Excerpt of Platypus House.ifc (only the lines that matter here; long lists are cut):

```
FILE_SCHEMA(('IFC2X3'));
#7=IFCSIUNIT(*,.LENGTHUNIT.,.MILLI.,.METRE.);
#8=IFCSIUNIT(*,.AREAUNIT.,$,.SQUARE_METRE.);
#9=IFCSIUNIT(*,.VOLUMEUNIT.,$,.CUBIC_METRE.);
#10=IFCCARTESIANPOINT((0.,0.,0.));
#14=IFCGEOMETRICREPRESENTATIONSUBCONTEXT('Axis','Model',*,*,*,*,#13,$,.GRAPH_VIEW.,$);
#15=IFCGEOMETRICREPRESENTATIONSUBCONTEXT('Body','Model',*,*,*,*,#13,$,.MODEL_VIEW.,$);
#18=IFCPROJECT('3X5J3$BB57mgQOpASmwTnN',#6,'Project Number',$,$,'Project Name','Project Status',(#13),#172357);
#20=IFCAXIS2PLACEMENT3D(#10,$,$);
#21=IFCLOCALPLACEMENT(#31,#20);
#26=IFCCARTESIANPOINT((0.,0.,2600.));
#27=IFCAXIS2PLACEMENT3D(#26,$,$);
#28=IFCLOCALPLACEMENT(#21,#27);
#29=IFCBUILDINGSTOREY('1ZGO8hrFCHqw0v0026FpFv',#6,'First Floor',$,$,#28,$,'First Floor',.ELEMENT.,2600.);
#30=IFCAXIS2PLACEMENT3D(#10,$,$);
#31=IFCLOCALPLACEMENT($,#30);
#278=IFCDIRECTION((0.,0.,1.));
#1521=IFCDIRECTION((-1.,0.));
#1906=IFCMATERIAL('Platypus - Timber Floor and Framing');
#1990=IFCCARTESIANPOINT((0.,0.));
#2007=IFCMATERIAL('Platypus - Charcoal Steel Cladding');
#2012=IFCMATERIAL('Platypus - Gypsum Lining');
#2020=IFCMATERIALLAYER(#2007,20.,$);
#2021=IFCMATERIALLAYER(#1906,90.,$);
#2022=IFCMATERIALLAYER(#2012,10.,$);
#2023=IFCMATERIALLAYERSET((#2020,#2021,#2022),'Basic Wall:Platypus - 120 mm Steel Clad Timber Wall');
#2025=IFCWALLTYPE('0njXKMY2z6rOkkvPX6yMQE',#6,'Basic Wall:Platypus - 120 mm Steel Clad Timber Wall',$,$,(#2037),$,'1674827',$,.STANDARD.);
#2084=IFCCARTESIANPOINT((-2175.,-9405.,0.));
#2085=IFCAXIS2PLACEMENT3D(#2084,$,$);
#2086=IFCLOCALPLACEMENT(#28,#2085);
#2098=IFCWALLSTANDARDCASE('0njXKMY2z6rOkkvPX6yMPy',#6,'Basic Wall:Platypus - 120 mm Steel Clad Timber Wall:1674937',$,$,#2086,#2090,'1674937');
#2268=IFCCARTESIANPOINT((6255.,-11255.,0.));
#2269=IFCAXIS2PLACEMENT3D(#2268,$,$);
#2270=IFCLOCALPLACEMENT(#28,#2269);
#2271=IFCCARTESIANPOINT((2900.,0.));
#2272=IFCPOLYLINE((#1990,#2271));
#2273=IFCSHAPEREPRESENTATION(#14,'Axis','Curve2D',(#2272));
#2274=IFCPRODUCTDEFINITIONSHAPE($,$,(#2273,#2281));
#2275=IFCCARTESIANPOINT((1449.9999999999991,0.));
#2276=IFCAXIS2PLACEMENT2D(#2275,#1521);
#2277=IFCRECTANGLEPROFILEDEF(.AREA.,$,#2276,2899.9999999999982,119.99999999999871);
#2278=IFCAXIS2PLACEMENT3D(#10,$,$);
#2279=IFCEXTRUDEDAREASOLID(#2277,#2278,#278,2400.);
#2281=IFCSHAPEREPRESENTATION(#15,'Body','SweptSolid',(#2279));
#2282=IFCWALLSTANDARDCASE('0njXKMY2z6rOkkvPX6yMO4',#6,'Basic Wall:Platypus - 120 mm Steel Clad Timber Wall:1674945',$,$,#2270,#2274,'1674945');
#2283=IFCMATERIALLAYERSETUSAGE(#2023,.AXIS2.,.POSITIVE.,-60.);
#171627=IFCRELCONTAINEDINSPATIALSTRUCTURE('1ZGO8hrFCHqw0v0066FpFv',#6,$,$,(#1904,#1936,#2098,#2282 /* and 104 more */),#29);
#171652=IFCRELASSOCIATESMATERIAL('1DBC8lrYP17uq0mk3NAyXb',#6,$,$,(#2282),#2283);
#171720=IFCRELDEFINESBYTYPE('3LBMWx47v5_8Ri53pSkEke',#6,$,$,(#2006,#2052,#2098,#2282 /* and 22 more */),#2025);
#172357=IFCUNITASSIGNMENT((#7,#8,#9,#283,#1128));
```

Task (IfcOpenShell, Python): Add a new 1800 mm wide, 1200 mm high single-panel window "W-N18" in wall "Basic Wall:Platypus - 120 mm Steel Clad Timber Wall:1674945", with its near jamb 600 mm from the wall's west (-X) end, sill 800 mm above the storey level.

```python
import numpy as np
import ifcopenshell
import ifcopenshell.api.feature
import ifcopenshell.api.geometry
import ifcopenshell.api.root
import ifcopenshell.api.spatial
import ifcopenshell.api.type
import ifcopenshell.geom
import ifcopenshell.util.element
import ifcopenshell.util.placement
import ifcopenshell.util.representation
import ifcopenshell.util.shape
import ifcopenshell.util.unit

model = ifcopenshell.open("Platypus House.ifc")
unit_scale = ifcopenshell.util.unit.calculate_unit_scale(model)
settings = ifcopenshell.geom.settings()


def volume(element):
    """Net volume in cubic metres, openings subtracted."""
    shape = ifcopenshell.geom.create_shape(settings, element)
    return ifcopenshell.util.shape.get_volume(shape.geometry)


wall = model.by_guid("0njXKMY2z6rOkkvPX6yMO4")
storey = ifcopenshell.util.element.get_container(wall, ifc_class="IfcBuildingStorey")
context = ifcopenshell.util.representation.get_context(model, "Model", "Body", "MODEL_VIEW")
before = volume(wall)

width, height, from_end, sill = 1.8, 1.2, 0.6, 0.8  # metres

# The wall runs along its own X axis, and the end named is its -X end.
wall_shape = ifcopenshell.geom.create_shape(settings, wall)
x, y, z = ifcopenshell.util.shape.get_vertices(wall_shape.geometry).T
start = x.min() + from_end
face, thickness = float(y.min()), float(y.max() - y.min())
wall_matrix = ifcopenshell.util.placement.get_local_placement(wall.ObjectPlacement)
level = ifcopenshell.util.placement.get_local_placement(storey.ObjectPlacement)[2, 3]


def in_wall(x, y):
    """Placement at x, y metres in the wall's axes, at sill height."""
    matrix = wall_matrix.copy()
    matrix[:, 3] = wall_matrix @ np.array([x / unit_scale, y / unit_scale, 0.0, 1.0])
    matrix[2, 3] = level + sill / unit_scale
    return matrix


# Opening: a box that overshoots both wall faces by 50 mm.
opening = ifcopenshell.api.root.create_entity(model, ifc_class="IfcOpeningElement")
box = ifcopenshell.api.geometry.add_wall_representation(
    model, context=context, length=width, height=height, thickness=thickness + 0.1
)
ifcopenshell.api.geometry.assign_representation(model, product=opening, representation=box)
ifcopenshell.api.geometry.edit_object_placement(model, product=opening, matrix=in_wall(start, face - 0.05), is_si=False)
ifcopenshell.api.feature.add_feature(model, feature=opening, element=wall)

window = ifcopenshell.api.root.create_entity(model, ifc_class="IfcWindow", name="W-N18")
window.OverallWidth, window.OverallHeight = width / unit_scale, height / unit_scale
body = ifcopenshell.api.geometry.add_window_representation(
    model,
    context=context,
    overall_width=window.OverallWidth,
    overall_height=window.OverallHeight,
    partition_type="SINGLE_PANEL",
)
ifcopenshell.api.geometry.assign_representation(model, product=window, representation=body)
ifcopenshell.api.spatial.assign_container(model, products=[window], relating_structure=storey)
fills = ifcopenshell.api.feature.add_filling(model, opening=opening, element=window)
fills.OwnerHistory = window.OwnerHistory  # required in IFC2X3

# IFC2X3 keeps the operation on the window style.
style = ifcopenshell.api.root.create_entity(model, ifc_class="IfcWindowStyle", name="W-N18")
style.OperationType, style.ConstructionType = "SINGLE_PANEL", "NOTDEFINED"
style.ParameterTakesPrecedence = style.Sizeable = False
ifcopenshell.api.type.assign_type(model, related_objects=[window], relating_type=style)

# Centre the window in the wall's thickness.
ifcopenshell.api.geometry.edit_object_placement(model, product=window, matrix=in_wall(start, face), is_si=False)
window_shape = ifcopenshell.geom.create_shape(settings, window)
depth = ifcopenshell.util.shape.get_vertices(window_shape.geometry)[:, 1]
offset = face + thickness / 2 - (depth.min() + depth.max()) / 2
ifcopenshell.api.geometry.edit_object_placement(model, product=window, matrix=in_wall(start, offset), is_si=False)

after = volume(wall)

print(f"wall volume {before:.3f} -> {after:.3f} m3")

model.write("Platypus House-out.ifc")
```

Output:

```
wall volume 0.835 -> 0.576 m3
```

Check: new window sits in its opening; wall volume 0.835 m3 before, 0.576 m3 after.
